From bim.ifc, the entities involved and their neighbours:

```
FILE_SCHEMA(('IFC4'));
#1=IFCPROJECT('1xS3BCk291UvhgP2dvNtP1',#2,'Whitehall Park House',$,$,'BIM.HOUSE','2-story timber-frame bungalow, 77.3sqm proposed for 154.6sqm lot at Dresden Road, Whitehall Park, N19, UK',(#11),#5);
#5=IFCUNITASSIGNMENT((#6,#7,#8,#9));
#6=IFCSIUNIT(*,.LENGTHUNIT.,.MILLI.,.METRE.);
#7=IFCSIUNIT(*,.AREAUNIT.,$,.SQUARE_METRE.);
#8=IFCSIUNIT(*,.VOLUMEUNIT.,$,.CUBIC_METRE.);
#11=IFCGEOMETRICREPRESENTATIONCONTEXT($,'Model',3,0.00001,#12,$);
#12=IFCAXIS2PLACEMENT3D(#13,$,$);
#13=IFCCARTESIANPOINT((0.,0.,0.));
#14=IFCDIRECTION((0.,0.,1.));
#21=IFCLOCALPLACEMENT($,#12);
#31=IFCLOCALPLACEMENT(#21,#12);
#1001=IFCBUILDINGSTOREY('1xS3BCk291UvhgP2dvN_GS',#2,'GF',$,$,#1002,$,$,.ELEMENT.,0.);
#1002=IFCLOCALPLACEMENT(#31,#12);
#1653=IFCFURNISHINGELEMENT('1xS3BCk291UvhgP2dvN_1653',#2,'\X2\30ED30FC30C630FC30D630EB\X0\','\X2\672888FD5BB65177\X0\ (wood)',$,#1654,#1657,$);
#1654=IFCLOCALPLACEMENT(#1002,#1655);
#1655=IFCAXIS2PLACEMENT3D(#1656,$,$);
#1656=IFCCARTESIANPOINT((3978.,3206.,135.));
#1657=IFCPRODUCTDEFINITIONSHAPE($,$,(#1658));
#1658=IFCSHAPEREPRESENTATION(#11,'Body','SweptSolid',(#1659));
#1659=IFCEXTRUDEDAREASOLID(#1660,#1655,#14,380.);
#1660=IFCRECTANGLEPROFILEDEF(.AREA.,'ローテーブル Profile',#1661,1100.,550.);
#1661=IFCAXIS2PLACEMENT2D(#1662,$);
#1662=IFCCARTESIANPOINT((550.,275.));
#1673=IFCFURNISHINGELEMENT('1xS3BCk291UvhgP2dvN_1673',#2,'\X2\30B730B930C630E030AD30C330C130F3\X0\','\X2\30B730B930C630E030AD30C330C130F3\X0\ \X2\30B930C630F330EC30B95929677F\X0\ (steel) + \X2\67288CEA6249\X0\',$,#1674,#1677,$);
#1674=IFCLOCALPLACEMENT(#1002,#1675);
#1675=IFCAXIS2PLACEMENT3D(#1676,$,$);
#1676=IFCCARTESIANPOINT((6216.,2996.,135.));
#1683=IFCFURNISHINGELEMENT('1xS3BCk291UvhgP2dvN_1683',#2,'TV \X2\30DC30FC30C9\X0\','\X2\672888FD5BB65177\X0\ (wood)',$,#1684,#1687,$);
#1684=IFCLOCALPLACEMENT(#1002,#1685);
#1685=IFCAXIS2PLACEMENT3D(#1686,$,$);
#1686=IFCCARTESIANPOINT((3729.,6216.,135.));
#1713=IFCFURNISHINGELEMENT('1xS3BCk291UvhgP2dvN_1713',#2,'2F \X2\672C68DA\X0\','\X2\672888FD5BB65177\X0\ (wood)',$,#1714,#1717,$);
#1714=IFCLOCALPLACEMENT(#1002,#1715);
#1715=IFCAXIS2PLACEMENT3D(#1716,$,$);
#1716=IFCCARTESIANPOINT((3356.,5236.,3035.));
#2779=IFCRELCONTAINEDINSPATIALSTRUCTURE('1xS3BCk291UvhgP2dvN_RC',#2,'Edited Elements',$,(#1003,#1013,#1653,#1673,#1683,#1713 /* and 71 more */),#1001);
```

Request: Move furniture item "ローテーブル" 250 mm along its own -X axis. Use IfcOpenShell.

```python
import ifcopenshell
import ifcopenshell.api.geometry
import ifcopenshell.util.placement
import ifcopenshell.util.unit

model = ifcopenshell.open("bim.ifc")
unit_scale = ifcopenshell.util.unit.calculate_unit_scale(model)

item = model.by_id(1653)
matrix = ifcopenshell.util.placement.get_local_placement(item.ObjectPlacement)
matrix[:3, 3] -= matrix[:3, 0] * 0.25 / unit_scale
ifcopenshell.api.geometry.edit_object_placement(model, product=item, matrix=matrix, is_si=False)

print(ifcopenshell.util.placement.get_local_placement(item.ObjectPlacement).round(3) + 0.0)

model.write("bim_v2.ifc")
```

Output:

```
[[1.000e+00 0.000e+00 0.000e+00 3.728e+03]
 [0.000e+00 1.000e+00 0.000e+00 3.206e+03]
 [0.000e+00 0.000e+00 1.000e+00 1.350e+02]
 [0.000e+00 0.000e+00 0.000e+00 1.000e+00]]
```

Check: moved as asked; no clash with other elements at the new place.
